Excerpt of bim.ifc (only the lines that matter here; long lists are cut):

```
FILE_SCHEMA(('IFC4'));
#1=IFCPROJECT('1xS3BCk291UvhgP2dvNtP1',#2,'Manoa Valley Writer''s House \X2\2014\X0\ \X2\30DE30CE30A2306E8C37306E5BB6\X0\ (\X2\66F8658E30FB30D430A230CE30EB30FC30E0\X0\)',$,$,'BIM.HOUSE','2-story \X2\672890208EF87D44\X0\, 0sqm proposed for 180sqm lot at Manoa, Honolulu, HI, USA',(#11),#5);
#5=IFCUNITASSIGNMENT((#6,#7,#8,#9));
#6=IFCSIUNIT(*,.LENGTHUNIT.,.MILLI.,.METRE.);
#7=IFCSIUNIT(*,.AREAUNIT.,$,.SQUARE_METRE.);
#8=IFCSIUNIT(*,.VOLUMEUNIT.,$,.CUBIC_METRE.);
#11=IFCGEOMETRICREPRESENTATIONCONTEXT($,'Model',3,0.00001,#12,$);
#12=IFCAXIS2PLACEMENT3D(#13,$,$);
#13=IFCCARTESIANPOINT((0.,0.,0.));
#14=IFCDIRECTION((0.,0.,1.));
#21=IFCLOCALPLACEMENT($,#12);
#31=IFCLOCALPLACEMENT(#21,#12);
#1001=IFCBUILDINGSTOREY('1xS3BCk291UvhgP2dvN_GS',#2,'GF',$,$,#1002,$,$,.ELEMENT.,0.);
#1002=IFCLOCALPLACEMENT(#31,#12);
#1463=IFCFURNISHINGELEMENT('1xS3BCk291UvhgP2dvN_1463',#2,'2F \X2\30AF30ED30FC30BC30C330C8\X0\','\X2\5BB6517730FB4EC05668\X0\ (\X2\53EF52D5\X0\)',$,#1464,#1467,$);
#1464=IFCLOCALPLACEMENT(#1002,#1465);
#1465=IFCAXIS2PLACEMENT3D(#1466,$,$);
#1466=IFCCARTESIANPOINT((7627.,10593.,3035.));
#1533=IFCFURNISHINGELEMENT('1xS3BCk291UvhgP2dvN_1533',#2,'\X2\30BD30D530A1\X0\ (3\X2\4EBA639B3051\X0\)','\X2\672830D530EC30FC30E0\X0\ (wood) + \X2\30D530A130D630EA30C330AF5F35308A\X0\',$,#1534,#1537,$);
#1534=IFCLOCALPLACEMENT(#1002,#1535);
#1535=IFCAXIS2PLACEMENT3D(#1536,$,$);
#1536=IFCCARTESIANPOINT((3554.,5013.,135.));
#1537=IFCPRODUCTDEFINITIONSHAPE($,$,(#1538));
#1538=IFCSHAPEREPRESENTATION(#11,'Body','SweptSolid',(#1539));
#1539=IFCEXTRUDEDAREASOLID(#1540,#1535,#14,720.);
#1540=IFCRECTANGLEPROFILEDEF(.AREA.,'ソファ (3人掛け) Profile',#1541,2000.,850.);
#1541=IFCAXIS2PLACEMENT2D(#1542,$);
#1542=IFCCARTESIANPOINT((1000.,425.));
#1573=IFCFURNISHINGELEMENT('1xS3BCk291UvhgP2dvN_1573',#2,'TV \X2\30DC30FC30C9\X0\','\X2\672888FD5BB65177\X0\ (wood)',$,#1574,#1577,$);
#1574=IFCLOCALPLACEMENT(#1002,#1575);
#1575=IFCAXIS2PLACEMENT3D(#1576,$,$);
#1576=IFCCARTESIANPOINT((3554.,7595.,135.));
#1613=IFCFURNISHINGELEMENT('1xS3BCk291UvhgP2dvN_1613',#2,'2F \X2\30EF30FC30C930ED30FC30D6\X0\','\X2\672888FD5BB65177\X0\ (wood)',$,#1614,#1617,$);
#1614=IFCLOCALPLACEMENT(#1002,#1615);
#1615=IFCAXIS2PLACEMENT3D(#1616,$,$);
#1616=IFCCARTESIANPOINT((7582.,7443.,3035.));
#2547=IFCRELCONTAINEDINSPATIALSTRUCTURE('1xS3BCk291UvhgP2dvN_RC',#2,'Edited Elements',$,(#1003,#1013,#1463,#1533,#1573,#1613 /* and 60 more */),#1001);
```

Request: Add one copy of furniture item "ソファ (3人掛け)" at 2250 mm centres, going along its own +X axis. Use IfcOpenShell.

```python
import ifcopenshell
import ifcopenshell.api.geometry
import ifcopenshell.api.root
import ifcopenshell.util.element
import ifcopenshell.util.placement
import ifcopenshell.util.unit

model = ifcopenshell.open("bim.ifc")
unit_scale = ifcopenshell.util.unit.calculate_unit_scale(model)


def reuse_history(source, copy):
    """copy_class also copies each property set's owner history, people and application; keep the originals."""
    for rel in copy.IsDefinedBy:
        if rel.is_a("IfcRelDefinesByProperties") and (history := rel.RelatingPropertyDefinition.OwnerHistory):
            rel.RelatingPropertyDefinition.OwnerHistory = source.OwnerHistory
            ifcopenshell.util.element.remove_deep2(model, history)


source = model.by_guid("1xS3BCk291UvhgP2dvN_1533")
base = ifcopenshell.util.placement.get_local_placement(source.ObjectPlacement)
step = base[:3, 0] * 2.25 / unit_scale

for i in range(1, 2):
    copy = ifcopenshell.api.root.copy_class(model, product=source)
    copy.Representation = ifcopenshell.util.element.copy_deep(
        model, source.Representation, exclude=["IfcGeometricRepresentationContext", "IfcRepresentationMap"]
    )
    reuse_history(source, copy)
    matrix = base.copy()
    matrix[:3, 3] += i * step
    print("added at", matrix[:3, 3].round(3) + 0.0)
    ifcopenshell.api.geometry.edit_object_placement(model, product=copy, matrix=matrix, is_si=False)

model.write("bim_rev.ifc")
```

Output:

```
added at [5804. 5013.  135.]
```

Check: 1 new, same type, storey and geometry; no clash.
